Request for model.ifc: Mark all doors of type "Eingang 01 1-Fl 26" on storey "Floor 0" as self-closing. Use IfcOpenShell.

First a look at what the model holds.

```python
import ifcopenshell
import ifcopenshell.util.element

model = ifcopenshell.open("model.ifc")
print(model.schema)
storey = next(s for s in model.by_type("IfcBuildingStorey") if s.Name == "Floor 0")
doors = [e for e in ifcopenshell.util.element.get_decomposition(storey) if e.is_a("IfcDoor")]
seen = {}
for e in doors:
    element_type = ifcopenshell.util.element.get_type(e)
    key = (element_type.Name if element_type != e and element_type else None, ifcopenshell.util.element.get_pset(e, "Pset_DoorCommon", "SelfClosing"))
    seen[key] = seen.get(key, 0) + 1
for (name, value), count in sorted(seen.items(), key=str):
    print(count, "x", name, "|", value)
```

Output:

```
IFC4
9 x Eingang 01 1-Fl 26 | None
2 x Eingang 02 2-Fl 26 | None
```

```python
import ifcopenshell
import ifcopenshell.api.pset
import ifcopenshell.util.element

model = ifcopenshell.open("model.ifc")

storey = next(s for s in model.by_type("IfcBuildingStorey") if s.Name == "Floor 0")
doors = [e for e in ifcopenshell.util.element.get_decomposition(storey) if e.is_a("IfcDoor")]

count = 0
for e in doors:
    element_type = ifcopenshell.util.element.get_type(e)
    if element_type in (None, e) or element_type.Name != "Eingang 01 1-Fl 26":
        continue
    # add_pset returns the element's existing set when there is one.
    pset = ifcopenshell.api.pset.add_pset(model, product=e, name="Pset_DoorCommon")
    ifcopenshell.api.pset.edit_pset(model, pset=pset, properties={"SelfClosing": True})
    count += 1

print(count, "doors updated")

model.write("model_v2.ifc")
```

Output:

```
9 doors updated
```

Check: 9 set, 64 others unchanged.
